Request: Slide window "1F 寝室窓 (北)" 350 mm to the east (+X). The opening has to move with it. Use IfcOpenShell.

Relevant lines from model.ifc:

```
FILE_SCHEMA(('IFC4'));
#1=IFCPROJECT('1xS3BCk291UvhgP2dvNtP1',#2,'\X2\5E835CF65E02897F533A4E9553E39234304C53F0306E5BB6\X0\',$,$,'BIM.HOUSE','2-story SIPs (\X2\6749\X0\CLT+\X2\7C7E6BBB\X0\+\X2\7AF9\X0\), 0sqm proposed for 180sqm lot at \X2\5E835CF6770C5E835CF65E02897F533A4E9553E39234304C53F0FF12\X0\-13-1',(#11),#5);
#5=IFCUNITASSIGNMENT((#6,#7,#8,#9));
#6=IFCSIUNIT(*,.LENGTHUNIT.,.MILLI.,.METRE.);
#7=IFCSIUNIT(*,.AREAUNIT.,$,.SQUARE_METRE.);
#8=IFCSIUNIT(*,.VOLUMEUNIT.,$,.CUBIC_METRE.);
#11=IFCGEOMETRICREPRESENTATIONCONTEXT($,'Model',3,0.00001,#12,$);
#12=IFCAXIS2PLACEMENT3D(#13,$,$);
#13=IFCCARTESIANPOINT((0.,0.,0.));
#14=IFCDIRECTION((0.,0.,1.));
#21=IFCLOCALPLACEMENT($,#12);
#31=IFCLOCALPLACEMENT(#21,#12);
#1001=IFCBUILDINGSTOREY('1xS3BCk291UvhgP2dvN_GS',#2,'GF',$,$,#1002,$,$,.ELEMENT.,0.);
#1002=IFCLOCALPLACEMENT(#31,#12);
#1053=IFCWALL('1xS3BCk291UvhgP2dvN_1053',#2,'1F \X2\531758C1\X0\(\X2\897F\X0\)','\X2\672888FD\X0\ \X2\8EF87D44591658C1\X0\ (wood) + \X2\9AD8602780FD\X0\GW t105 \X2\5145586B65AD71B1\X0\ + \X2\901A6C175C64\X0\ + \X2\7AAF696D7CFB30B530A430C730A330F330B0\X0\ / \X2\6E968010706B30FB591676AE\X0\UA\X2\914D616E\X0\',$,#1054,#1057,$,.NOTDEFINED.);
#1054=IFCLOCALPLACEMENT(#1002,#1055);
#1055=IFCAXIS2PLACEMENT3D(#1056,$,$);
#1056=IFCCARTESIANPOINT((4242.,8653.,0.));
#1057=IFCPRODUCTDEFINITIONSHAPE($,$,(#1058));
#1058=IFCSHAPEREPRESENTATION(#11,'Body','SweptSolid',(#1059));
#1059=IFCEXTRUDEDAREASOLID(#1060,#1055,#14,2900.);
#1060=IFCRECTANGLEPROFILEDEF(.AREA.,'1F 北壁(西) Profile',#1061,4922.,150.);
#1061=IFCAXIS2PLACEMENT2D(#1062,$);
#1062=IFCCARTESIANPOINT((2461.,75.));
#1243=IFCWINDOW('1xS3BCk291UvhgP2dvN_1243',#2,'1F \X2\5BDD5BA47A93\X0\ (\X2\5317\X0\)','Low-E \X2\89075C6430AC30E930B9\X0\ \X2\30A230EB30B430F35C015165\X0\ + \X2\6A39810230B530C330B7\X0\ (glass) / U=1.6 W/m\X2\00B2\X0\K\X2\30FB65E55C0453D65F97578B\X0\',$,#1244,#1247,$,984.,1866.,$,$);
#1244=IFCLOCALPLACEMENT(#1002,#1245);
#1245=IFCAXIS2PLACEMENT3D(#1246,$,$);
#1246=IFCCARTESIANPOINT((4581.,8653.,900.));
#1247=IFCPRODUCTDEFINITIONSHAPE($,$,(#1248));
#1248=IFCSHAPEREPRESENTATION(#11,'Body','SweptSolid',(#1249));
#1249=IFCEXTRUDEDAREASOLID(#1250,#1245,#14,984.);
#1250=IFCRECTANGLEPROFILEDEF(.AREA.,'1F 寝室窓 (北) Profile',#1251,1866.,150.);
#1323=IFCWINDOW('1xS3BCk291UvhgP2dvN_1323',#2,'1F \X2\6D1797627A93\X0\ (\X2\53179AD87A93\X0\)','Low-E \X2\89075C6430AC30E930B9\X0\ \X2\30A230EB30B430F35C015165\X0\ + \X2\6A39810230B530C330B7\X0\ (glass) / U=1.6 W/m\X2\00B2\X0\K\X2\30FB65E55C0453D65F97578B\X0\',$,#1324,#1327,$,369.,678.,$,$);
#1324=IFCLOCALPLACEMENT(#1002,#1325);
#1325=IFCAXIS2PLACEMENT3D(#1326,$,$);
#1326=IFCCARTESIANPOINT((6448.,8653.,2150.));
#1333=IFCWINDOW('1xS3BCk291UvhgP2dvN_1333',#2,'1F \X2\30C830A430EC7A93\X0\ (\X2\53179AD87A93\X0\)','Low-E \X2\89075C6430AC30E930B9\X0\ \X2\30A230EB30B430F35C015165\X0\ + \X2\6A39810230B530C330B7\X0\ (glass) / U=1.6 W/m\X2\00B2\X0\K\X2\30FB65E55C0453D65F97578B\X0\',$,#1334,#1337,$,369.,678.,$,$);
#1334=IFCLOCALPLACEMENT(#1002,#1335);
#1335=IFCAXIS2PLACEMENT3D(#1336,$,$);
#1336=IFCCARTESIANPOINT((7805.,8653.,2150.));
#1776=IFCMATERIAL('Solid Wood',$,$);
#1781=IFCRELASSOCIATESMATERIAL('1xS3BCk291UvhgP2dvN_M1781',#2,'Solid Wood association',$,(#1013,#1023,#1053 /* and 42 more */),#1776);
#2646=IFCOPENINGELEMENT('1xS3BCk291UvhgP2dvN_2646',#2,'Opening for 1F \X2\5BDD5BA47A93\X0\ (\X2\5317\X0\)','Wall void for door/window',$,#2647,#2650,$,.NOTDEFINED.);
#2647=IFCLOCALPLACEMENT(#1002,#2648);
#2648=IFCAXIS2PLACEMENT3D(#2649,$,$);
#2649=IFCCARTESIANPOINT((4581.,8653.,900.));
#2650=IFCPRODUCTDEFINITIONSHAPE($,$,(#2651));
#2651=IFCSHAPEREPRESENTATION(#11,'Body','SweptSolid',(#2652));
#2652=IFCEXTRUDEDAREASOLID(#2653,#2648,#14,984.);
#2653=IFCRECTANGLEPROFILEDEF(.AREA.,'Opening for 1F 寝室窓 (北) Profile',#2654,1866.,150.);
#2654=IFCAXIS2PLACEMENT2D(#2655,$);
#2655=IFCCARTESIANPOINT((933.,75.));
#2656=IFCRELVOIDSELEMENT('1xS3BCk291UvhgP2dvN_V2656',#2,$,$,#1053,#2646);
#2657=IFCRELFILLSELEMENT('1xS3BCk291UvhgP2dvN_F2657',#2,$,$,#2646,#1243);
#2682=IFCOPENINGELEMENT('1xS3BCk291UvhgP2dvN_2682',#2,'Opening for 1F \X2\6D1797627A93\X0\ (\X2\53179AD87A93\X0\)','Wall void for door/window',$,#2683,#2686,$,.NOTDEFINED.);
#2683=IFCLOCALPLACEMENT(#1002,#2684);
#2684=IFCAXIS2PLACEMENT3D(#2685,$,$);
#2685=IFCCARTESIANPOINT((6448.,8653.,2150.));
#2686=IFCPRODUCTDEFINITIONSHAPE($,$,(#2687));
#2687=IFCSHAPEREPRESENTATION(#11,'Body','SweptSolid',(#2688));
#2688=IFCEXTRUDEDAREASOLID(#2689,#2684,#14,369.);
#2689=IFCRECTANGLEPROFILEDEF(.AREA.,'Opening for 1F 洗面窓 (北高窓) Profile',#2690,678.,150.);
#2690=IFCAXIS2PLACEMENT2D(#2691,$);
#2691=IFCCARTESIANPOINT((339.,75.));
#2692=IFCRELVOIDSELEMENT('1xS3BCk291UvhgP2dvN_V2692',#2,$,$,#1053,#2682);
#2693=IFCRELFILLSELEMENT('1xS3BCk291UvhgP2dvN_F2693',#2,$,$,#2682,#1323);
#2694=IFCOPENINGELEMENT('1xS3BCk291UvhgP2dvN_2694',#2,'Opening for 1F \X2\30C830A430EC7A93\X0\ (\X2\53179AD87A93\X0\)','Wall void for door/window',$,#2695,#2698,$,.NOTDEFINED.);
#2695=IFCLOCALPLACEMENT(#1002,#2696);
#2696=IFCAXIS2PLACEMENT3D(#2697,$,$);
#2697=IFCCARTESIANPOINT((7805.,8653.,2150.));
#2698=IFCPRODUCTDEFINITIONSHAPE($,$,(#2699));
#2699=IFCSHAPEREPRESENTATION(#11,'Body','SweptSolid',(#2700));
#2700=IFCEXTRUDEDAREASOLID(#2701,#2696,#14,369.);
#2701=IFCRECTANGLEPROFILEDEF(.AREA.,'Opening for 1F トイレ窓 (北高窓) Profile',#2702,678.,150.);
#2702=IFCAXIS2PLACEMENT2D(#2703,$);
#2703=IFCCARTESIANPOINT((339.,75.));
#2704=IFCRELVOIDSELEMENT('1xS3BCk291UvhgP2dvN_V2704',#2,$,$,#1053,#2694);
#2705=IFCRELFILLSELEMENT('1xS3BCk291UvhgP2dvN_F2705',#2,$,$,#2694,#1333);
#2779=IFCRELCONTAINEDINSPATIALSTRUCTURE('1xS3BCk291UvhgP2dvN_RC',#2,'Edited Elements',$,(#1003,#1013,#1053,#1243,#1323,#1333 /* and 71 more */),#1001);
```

```python
import ifcopenshell
import ifcopenshell.api.geometry
import ifcopenshell.util.placement
import ifcopenshell.util.unit

model = ifcopenshell.open("model.ifc")
unit_scale = ifcopenshell.util.unit.calculate_unit_scale(model)

window = model.by_guid("1xS3BCk291UvhgP2dvN_1243")
opening = window.FillsVoids[0].RelatingOpeningElement
wall = opening.VoidsElements[0].RelatingBuildingElement

wall_matrix = ifcopenshell.util.placement.get_local_placement(wall.ObjectPlacement)
shift = wall_matrix[:3, 0] * 0.35 / unit_scale
before = ifcopenshell.util.placement.get_local_placement(window.ObjectPlacement)[:3, 3].copy()

# The window is not placed relative to its opening, so move both.
for product in (opening, window):
    matrix = ifcopenshell.util.placement.get_local_placement(product.ObjectPlacement)
    matrix[:3, 3] += shift
    ifcopenshell.api.geometry.edit_object_placement(model, product=product, matrix=matrix, is_si=False)

after = ifcopenshell.util.placement.get_local_placement(window.ObjectPlacement)[:3, 3]
print("window moved by", (after - before).round(3) + 0.0)

model.write("model_updated.ifc")
```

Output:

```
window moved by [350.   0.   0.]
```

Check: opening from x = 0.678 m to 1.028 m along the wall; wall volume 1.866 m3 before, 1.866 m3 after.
